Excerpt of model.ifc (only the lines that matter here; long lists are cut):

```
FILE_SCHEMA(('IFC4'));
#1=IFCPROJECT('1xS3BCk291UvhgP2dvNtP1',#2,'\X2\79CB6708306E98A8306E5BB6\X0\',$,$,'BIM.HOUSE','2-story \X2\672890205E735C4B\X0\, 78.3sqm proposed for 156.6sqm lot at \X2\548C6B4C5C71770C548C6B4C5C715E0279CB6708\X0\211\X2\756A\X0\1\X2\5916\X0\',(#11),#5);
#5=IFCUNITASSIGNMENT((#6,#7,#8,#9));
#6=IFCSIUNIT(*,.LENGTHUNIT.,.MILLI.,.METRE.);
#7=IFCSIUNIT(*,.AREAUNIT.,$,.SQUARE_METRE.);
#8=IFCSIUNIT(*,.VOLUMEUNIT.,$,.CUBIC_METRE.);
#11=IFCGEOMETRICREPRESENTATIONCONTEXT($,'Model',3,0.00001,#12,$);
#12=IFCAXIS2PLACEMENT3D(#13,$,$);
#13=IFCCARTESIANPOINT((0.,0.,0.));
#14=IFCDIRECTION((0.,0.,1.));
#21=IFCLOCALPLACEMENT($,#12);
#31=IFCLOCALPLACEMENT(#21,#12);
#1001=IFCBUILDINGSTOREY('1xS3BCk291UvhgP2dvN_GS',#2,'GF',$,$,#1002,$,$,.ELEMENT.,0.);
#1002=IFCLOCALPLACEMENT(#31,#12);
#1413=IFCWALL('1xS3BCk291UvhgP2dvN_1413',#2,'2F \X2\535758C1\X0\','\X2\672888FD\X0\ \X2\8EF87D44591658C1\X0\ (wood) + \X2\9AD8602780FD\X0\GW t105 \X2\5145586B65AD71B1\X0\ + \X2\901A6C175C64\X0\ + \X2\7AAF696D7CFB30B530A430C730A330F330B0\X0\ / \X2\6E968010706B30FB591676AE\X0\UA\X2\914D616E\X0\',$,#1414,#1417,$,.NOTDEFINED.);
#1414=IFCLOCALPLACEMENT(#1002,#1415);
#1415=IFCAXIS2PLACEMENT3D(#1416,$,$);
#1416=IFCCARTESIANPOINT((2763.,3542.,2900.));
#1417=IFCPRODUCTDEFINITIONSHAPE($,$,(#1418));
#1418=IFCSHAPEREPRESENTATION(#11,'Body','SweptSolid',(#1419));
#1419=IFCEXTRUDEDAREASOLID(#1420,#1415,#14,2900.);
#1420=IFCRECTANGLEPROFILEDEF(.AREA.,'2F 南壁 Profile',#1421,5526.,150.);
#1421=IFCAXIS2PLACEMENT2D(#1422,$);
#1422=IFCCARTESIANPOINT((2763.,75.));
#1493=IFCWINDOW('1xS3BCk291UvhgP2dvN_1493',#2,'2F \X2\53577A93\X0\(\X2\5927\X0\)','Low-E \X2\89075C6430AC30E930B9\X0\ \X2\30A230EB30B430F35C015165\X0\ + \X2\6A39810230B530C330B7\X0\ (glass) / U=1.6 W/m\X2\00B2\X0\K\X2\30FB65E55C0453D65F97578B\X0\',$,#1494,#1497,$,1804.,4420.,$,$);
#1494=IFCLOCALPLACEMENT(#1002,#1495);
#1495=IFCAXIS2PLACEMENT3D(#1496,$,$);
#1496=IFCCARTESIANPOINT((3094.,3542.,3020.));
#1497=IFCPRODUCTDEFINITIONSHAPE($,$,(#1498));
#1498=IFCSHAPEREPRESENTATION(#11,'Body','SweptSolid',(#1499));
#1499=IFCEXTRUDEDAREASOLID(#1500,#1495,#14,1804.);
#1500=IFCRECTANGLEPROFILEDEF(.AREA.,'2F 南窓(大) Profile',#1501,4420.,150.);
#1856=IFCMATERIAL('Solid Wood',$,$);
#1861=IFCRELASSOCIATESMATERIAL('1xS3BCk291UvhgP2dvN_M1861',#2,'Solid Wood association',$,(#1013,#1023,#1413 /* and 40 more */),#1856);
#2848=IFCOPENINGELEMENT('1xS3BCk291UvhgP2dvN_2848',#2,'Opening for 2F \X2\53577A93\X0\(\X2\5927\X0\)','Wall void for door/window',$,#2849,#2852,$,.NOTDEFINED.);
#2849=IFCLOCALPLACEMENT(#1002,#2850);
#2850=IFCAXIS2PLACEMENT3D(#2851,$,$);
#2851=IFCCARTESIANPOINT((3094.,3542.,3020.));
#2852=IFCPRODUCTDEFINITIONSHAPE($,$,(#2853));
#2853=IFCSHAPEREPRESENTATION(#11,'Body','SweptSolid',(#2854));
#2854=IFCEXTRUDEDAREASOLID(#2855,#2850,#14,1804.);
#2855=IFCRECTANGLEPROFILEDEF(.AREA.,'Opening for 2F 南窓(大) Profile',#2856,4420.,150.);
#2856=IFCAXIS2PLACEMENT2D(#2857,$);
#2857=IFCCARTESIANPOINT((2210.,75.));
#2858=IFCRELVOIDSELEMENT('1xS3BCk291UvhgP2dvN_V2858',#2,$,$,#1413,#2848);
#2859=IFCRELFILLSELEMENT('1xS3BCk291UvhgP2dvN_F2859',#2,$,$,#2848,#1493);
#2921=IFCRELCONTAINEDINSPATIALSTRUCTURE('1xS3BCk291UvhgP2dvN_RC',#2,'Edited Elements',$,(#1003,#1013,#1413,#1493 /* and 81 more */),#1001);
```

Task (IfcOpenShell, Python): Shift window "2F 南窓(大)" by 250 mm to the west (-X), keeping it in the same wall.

```python
import ifcopenshell
import ifcopenshell.api.geometry
import ifcopenshell.util.placement
import ifcopenshell.util.unit

model = ifcopenshell.open("model.ifc")
unit_scale = ifcopenshell.util.unit.calculate_unit_scale(model)

window = model.by_guid("1xS3BCk291UvhgP2dvN_1493")
opening = window.FillsVoids[0].RelatingOpeningElement
wall = opening.VoidsElements[0].RelatingBuildingElement

wall_matrix = ifcopenshell.util.placement.get_local_placement(wall.ObjectPlacement)
shift = wall_matrix[:3, 0] * -0.25 / unit_scale
before = ifcopenshell.util.placement.get_local_placement(window.ObjectPlacement)[:3, 3].copy()

# The window is not placed relative to its opening, so move both.
for product in (opening, window):
    matrix = ifcopenshell.util.placement.get_local_placement(product.ObjectPlacement)
    matrix[:3, 3] += shift
    ifcopenshell.api.geometry.edit_object_placement(model, product=product, matrix=matrix, is_si=False)

after = ifcopenshell.util.placement.get_local_placement(window.ObjectPlacement)[:3, 3]
print("window moved by", (after - before).round(3) + 0.0)

model.write("model_updated.ifc")
```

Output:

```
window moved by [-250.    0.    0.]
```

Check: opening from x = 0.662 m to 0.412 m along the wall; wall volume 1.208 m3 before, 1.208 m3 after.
